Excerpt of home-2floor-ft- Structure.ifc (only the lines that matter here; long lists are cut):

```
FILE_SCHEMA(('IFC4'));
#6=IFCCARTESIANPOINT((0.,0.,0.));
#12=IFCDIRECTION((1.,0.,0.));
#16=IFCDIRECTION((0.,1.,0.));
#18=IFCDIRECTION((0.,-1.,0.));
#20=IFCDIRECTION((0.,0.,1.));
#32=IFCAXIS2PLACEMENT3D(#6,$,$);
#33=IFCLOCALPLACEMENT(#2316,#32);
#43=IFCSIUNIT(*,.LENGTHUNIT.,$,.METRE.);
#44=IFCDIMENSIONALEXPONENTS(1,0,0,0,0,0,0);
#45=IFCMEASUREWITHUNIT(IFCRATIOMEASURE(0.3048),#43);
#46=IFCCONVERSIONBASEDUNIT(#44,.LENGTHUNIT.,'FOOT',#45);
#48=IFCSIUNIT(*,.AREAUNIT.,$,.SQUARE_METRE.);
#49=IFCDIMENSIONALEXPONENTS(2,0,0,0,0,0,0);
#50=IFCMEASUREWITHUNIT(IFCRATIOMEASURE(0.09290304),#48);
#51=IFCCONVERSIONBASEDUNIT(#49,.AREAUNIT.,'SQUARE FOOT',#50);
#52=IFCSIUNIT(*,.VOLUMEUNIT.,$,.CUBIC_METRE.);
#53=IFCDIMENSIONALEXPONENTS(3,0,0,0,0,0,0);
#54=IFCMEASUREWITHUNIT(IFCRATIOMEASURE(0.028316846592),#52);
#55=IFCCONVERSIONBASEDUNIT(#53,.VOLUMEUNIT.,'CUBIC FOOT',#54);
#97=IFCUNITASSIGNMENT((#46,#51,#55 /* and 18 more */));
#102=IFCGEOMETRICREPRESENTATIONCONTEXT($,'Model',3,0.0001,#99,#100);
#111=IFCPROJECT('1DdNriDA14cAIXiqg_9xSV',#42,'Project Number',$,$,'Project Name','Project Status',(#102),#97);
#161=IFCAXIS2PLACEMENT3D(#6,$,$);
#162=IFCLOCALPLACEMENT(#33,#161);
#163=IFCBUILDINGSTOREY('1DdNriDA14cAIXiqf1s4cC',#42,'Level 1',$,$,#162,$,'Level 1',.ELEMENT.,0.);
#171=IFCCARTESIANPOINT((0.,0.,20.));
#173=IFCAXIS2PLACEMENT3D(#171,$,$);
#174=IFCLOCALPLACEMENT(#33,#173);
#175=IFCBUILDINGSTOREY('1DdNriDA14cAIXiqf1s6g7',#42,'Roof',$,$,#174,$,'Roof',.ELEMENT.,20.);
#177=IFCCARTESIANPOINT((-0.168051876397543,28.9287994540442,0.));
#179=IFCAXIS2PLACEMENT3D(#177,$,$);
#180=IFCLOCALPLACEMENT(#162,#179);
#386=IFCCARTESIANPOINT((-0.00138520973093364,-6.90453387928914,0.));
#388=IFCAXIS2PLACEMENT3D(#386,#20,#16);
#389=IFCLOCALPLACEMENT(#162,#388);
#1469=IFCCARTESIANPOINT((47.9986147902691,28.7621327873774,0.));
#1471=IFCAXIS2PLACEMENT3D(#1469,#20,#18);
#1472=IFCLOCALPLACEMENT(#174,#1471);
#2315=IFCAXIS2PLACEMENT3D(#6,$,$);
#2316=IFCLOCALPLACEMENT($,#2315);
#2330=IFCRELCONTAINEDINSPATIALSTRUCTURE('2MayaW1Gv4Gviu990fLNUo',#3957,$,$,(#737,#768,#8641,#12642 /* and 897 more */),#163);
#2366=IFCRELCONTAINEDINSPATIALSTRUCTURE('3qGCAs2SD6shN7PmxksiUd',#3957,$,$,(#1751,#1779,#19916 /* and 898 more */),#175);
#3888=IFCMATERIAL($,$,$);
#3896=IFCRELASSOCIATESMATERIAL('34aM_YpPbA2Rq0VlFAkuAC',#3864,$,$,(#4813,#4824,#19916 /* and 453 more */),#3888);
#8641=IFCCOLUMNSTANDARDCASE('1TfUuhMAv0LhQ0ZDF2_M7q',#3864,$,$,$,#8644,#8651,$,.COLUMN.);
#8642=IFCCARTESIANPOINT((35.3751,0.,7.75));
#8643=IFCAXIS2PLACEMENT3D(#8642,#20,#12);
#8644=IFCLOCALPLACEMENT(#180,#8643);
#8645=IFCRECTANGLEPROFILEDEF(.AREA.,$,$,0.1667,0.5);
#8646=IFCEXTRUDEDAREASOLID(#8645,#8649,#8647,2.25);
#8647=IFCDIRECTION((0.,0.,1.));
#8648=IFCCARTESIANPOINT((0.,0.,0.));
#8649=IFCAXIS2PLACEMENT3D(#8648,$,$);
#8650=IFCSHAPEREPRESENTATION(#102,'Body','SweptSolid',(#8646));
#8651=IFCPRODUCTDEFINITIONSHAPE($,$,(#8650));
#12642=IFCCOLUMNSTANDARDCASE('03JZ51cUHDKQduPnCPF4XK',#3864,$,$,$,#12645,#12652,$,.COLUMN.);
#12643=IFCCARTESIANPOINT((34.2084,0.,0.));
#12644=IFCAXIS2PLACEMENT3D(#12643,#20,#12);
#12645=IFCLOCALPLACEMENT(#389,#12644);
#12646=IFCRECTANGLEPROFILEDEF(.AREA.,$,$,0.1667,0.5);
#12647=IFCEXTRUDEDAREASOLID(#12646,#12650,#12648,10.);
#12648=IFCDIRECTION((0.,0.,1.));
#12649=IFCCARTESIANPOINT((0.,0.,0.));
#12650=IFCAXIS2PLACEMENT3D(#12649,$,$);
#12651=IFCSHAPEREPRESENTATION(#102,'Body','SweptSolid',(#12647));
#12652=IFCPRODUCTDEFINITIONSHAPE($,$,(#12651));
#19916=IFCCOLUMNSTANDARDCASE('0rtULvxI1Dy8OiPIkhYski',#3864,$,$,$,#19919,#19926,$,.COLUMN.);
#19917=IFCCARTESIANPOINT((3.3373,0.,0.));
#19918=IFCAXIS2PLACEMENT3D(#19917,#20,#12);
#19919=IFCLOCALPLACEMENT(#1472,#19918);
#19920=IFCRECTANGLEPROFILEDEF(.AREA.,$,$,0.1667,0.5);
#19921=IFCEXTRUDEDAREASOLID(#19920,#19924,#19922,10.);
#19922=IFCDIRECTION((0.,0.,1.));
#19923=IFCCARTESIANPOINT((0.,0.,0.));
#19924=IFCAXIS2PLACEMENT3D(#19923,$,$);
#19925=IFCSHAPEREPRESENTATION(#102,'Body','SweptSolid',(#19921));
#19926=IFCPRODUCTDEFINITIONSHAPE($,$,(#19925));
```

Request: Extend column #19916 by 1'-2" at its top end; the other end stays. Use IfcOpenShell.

```python
import ifcopenshell
import ifcopenshell.util.unit

model = ifcopenshell.open("home-2floor-ft- Structure.ifc")
unit_scale = ifcopenshell.util.unit.calculate_unit_scale(model)

member = model.by_guid("0rtULvxI1Dy8OiPIkhYski")
change = 14 * 0.0254 / unit_scale

# The extrusion runs towards the end named, so only its depth changes.
body = next(r for r in member.Representation.Representations if r.RepresentationIdentifier == "Body")
solid = body.Items[0]
old_length = solid.Depth
solid.Depth += change

print(f"length {old_length:g} -> {solid.Depth:g}")

model.write("home-2floor-ft- Structure-out.ifc")
```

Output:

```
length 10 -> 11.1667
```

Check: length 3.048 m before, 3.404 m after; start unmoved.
